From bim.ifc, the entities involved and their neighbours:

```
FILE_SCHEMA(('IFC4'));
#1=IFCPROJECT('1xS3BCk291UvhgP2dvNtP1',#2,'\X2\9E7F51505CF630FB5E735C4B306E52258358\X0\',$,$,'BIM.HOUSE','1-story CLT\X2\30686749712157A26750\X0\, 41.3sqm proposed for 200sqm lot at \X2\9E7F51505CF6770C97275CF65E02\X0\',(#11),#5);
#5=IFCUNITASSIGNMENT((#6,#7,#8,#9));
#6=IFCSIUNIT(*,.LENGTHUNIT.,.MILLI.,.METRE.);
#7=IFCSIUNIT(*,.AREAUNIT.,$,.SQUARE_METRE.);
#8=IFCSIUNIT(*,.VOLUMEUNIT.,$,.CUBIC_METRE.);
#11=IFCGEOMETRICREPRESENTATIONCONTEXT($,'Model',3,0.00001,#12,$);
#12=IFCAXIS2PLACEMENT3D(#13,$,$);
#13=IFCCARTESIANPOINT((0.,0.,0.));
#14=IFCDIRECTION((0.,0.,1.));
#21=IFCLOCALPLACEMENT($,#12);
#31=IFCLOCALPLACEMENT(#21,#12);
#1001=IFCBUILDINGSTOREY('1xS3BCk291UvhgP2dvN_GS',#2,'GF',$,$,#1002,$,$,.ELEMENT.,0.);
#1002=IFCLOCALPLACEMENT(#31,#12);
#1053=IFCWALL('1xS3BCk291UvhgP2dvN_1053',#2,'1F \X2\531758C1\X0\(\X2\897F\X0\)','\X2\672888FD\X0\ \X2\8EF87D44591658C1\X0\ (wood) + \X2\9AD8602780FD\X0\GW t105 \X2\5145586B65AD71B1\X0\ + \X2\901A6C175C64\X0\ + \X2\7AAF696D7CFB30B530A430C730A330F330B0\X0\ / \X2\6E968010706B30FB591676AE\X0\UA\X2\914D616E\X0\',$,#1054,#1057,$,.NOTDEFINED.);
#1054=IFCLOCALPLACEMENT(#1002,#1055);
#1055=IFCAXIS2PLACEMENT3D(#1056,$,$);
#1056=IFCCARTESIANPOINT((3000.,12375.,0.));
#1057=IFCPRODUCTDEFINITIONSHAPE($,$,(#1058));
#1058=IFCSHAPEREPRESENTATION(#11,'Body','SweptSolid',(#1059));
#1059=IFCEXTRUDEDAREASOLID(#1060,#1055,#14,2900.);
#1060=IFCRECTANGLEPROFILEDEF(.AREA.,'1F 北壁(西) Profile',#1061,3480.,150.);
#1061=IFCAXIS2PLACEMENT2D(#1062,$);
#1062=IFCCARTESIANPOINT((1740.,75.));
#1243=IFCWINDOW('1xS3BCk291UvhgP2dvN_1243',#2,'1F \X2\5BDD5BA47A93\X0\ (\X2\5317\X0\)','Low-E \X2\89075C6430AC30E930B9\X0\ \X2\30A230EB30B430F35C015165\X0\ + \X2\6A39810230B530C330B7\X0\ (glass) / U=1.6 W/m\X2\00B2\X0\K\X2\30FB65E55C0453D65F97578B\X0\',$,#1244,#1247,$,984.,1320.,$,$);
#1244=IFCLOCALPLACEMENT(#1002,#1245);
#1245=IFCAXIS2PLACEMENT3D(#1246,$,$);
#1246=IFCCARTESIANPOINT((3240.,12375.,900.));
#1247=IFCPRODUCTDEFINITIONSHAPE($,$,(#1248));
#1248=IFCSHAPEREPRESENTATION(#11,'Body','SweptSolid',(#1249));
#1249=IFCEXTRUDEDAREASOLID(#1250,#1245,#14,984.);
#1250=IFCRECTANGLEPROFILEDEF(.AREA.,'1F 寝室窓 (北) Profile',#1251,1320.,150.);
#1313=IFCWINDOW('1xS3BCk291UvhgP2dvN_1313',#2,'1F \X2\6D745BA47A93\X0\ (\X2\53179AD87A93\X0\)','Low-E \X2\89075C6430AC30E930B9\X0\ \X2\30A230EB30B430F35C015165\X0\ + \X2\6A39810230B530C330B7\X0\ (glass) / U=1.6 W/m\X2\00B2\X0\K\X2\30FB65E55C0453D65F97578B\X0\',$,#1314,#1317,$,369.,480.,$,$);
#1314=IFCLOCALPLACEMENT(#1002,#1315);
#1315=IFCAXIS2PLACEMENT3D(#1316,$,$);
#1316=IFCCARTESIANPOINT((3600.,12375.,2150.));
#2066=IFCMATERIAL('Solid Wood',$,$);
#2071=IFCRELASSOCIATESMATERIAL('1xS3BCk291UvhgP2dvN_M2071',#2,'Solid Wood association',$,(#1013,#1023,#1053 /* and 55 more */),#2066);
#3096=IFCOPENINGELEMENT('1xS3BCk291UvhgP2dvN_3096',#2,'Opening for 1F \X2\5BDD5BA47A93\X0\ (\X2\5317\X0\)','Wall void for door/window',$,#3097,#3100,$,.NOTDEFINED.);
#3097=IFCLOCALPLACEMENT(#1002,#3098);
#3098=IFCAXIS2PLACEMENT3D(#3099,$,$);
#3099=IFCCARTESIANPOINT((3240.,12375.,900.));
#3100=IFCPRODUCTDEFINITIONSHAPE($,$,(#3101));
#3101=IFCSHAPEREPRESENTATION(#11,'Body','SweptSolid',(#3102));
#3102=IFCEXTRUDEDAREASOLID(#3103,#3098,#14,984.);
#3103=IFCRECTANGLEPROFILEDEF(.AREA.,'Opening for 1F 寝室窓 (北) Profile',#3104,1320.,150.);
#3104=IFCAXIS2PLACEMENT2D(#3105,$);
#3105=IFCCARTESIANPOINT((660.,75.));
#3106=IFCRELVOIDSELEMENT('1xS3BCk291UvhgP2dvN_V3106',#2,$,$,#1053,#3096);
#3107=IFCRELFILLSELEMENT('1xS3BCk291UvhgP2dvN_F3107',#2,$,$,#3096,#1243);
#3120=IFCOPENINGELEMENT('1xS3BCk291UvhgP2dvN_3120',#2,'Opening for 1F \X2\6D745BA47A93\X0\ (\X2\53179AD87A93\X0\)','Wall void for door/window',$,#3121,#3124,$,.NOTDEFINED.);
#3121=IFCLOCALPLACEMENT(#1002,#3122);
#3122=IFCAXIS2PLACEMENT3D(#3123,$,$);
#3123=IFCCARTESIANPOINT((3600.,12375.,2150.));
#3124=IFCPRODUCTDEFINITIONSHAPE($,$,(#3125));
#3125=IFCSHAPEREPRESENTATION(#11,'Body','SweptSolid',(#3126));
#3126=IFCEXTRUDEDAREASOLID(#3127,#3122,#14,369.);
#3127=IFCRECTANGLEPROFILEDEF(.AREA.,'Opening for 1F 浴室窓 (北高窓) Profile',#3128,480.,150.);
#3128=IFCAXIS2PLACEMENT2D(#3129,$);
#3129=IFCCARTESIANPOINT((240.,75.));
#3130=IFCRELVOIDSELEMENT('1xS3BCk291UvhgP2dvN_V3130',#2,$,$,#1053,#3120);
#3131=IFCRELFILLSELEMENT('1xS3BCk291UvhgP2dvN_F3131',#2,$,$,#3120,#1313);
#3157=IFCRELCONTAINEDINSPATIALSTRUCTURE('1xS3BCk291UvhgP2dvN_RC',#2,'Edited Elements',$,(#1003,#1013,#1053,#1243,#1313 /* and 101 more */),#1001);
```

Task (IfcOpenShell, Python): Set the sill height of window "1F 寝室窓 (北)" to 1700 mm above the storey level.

```python
import numpy as np
import ifcopenshell
import ifcopenshell.api.geometry
import ifcopenshell.geom
import ifcopenshell.util.element
import ifcopenshell.util.placement
import ifcopenshell.util.shape
import ifcopenshell.util.unit

model = ifcopenshell.open("bim.ifc")
unit_scale = ifcopenshell.util.unit.calculate_unit_scale(model)

window = model.by_id(1243)
opening = window.FillsVoids[0].RelatingOpeningElement
storey = ifcopenshell.util.element.get_container(window, ifc_class="IfcBuildingStorey")
level = ifcopenshell.util.placement.get_local_placement(storey.ObjectPlacement)[2, 3]

# The opening's origin need not be at the sill, so measure its lowest point.
shape = ifcopenshell.geom.create_shape(ifcopenshell.geom.settings(), opening)
bottom = ifcopenshell.util.shape.get_shape_bottom_elevation(shape, shape.geometry) / unit_scale
dz = level + 1.7 / unit_scale - bottom

shift = np.array([0.0, 0.0, dz])
# The window is not placed relative to its opening, so move both.
for product in (opening, window):
    matrix = ifcopenshell.util.placement.get_local_placement(product.ObjectPlacement)
    matrix[:3, 3] += shift
    ifcopenshell.api.geometry.edit_object_placement(model, product=product, matrix=matrix, is_si=False)

print(f"moved by {dz * unit_scale:+.3f} m")

model.write("bim_v2.ifc")
```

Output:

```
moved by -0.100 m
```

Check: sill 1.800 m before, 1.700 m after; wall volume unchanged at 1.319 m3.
